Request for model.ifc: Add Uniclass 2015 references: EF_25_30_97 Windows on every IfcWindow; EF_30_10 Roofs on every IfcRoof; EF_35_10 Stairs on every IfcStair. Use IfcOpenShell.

First a look at what the model holds.

```python
import ifcopenshell

model = ifcopenshell.open("model.ifc")
print(model.schema)
print("classifications:", [c.Name for c in model.by_type("IfcClassification")])
for ifc_class in ("IfcDoor", "IfcRoof", "IfcStair", "IfcWall", "IfcWindow"):
    print(ifc_class, len(model.by_type(ifc_class)))
```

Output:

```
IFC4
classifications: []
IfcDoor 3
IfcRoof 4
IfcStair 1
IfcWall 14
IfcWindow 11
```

```python
import ifcopenshell
import ifcopenshell.api.classification

model = ifcopenshell.open("model.ifc")

system = ifcopenshell.api.classification.add_classification(model, classification="Uniclass 2015")

codes = {
    "IfcWindow": ("EF_25_30_97", "Windows"),
    "IfcRoof": ("EF_30_10", "Roofs"),
    "IfcStair": ("EF_35_10", "Stairs"),
}
for ifc_class, (code, name) in codes.items():
    products = model.by_type(ifc_class)
    ifcopenshell.api.classification.add_reference(
        model, products=products, classification=system, identification=code, name=name
    )
    print(code, len(products))

model.write("model_edited.ifc")
```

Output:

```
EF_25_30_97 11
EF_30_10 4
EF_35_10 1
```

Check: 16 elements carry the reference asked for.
